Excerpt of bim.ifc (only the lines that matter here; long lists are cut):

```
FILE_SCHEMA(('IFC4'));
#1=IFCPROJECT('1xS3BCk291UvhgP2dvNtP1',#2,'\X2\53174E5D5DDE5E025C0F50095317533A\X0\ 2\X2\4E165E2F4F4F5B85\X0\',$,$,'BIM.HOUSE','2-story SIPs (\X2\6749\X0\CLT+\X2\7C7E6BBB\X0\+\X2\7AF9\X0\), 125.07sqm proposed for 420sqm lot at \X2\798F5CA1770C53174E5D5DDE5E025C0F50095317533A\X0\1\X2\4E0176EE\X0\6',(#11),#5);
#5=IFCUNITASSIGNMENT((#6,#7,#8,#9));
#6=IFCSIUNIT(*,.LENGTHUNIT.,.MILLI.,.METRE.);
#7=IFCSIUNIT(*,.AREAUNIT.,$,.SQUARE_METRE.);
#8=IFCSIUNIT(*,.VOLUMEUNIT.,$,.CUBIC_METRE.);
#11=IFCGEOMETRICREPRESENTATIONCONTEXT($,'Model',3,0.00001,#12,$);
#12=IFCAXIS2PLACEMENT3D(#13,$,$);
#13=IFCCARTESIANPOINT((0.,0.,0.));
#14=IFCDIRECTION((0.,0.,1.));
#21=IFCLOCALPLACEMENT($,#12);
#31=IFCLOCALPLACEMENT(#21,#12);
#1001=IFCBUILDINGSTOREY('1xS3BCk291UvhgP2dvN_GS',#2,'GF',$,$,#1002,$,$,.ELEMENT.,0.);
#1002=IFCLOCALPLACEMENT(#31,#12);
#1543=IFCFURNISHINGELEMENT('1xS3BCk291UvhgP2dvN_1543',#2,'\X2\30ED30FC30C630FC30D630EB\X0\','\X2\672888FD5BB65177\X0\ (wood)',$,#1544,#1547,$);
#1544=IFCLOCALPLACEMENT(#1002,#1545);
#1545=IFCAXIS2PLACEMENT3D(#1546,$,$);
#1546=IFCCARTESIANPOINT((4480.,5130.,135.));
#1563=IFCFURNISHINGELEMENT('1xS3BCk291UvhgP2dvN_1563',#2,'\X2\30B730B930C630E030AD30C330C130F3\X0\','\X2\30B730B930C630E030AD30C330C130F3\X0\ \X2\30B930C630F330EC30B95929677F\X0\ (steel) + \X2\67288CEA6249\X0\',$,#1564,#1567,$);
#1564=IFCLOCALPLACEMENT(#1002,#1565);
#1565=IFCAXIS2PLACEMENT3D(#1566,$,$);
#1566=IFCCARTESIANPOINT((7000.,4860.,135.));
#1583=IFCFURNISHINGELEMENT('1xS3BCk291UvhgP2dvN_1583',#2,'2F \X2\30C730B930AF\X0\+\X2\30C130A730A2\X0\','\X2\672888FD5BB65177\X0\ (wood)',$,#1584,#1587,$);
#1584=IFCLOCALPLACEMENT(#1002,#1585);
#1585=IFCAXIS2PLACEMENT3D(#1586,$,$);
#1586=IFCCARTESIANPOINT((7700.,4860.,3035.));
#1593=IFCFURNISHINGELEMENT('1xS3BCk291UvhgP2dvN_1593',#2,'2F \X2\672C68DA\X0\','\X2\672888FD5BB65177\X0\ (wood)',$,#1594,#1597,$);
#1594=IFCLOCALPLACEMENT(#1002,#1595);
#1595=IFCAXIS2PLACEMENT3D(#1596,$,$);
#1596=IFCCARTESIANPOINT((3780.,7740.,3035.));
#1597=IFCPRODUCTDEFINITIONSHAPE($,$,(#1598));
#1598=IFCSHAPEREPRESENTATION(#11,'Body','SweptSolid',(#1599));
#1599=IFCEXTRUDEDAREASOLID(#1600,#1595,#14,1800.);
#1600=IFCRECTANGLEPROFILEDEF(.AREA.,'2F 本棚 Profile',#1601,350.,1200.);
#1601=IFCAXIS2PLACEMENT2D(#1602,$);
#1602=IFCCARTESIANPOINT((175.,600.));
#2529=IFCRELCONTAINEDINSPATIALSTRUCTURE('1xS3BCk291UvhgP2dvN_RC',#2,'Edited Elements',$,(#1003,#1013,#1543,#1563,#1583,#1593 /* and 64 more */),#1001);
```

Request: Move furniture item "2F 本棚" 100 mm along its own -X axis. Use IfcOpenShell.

```python
import ifcopenshell
import ifcopenshell.api.geometry
import ifcopenshell.util.placement
import ifcopenshell.util.unit

model = ifcopenshell.open("bim.ifc")
unit_scale = ifcopenshell.util.unit.calculate_unit_scale(model)

item = model.by_guid("1xS3BCk291UvhgP2dvN_1593")
matrix = ifcopenshell.util.placement.get_local_placement(item.ObjectPlacement)
matrix[:3, 3] -= matrix[:3, 0] * 0.1 / unit_scale
ifcopenshell.api.geometry.edit_object_placement(model, product=item, matrix=matrix, is_si=False)

print(ifcopenshell.util.placement.get_local_placement(item.ObjectPlacement).round(3) + 0.0)

model.write("bim_edited.ifc")
```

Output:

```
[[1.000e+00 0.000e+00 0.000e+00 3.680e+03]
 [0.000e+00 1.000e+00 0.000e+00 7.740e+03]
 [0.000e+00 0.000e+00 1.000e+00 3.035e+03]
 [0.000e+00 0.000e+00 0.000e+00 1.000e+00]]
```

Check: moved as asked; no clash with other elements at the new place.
